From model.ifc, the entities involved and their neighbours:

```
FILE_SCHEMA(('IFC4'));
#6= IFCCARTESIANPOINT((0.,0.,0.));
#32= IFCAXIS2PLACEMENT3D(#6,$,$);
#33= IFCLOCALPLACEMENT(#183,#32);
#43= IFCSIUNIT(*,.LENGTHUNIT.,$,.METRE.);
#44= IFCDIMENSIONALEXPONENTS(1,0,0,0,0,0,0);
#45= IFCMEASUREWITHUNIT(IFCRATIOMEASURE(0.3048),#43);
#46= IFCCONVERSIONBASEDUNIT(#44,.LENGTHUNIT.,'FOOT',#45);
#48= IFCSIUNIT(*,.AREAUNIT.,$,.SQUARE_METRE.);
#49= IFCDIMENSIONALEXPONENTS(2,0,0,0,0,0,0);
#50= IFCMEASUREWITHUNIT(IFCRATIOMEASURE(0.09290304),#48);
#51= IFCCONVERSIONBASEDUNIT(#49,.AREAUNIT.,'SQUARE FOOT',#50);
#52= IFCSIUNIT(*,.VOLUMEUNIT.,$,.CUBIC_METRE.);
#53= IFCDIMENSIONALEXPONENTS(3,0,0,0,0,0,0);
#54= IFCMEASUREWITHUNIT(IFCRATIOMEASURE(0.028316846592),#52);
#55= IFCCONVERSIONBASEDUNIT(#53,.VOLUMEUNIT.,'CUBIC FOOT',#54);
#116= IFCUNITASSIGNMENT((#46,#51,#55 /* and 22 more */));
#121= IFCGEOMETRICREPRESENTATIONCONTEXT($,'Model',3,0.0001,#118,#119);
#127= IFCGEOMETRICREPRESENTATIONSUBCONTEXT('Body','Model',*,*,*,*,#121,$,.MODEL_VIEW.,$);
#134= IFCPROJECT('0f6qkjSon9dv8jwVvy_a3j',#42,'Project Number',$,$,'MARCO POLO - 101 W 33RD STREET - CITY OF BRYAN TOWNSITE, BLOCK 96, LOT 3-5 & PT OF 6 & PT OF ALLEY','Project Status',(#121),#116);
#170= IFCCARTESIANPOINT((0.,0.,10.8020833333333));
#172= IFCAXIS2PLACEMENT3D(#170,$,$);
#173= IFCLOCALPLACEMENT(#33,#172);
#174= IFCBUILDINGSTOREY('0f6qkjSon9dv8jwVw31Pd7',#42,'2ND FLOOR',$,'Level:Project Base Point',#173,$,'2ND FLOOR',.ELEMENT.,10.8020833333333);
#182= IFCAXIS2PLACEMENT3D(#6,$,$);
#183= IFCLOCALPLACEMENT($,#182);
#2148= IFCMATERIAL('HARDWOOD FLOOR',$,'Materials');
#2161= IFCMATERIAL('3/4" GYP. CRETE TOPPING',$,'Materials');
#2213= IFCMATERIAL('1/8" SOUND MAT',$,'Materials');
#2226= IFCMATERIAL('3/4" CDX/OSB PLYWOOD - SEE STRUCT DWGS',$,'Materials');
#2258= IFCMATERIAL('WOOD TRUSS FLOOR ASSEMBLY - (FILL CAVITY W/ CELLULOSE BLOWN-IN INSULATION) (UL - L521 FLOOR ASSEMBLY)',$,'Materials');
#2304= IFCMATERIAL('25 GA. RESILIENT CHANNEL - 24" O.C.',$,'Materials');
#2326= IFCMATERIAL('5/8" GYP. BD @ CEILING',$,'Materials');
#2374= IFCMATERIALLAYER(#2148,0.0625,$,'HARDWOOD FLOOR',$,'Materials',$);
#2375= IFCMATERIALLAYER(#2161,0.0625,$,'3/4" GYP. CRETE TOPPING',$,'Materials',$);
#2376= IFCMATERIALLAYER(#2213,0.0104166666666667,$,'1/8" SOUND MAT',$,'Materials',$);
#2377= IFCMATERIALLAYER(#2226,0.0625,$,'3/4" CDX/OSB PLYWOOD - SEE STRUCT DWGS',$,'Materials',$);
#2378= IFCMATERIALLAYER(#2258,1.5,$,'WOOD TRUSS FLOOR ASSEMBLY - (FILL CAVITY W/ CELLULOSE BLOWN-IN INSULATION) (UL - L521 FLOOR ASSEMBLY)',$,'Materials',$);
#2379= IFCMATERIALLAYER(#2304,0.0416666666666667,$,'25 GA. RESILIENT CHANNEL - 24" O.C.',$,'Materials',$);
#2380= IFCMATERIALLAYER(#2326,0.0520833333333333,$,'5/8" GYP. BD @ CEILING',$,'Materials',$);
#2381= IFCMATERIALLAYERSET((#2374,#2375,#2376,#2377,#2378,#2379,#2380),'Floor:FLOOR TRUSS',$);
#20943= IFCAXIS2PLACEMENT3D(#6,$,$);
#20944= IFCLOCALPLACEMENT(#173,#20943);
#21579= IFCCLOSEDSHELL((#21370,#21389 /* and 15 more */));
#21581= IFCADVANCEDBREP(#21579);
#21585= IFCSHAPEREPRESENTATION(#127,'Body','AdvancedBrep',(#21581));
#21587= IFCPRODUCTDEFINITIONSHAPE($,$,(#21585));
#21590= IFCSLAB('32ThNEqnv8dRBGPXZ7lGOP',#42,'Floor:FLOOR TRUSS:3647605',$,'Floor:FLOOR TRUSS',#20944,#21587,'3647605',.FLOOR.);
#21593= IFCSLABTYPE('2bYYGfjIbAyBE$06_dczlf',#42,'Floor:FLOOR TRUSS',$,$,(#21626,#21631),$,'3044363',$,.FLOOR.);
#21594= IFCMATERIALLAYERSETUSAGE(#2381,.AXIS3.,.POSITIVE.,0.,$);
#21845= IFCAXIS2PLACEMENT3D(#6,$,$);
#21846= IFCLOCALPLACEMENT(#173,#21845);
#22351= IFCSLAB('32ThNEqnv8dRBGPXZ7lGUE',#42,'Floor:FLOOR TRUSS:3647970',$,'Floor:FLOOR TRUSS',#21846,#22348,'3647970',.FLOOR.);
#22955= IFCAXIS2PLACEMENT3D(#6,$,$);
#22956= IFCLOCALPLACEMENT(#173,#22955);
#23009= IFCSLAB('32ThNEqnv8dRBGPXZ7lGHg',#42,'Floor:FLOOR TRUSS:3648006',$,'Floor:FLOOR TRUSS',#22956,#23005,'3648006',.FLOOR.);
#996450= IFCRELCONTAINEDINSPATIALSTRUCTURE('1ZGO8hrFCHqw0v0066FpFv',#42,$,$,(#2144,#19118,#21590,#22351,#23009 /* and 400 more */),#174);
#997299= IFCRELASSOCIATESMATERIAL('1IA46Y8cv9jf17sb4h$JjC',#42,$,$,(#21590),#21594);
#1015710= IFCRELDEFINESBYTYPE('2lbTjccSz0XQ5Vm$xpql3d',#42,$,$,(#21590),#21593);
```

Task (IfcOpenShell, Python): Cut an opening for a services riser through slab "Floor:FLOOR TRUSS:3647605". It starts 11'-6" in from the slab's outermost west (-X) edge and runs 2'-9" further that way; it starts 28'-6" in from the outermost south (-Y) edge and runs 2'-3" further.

```python
import numpy as np
import ifcopenshell
import ifcopenshell.api.feature
import ifcopenshell.api.geometry
import ifcopenshell.api.root
import ifcopenshell.geom
import ifcopenshell.util.placement
import ifcopenshell.util.representation
import ifcopenshell.util.shape
import ifcopenshell.util.unit

model = ifcopenshell.open("model.ifc")
unit_scale = ifcopenshell.util.unit.calculate_unit_scale(model)
settings = ifcopenshell.geom.settings()


def volume(element):
    """Net volume in cubic metres, openings subtracted."""
    shape = ifcopenshell.geom.create_shape(settings, element)
    return ifcopenshell.util.shape.get_volume(shape.geometry)


slab = model.by_guid("32ThNEqnv8dRBGPXZ7lGOP")
before = volume(slab)

# Extent in the slab's own axes, in metres. The edges named are its -X and -Y sides.
slab_shape = ifcopenshell.geom.create_shape(settings, slab)
vertices = ifcopenshell.util.shape.get_vertices(slab_shape.geometry)
x_min, y_min, bottom = vertices.min(axis=0)
top = vertices[:, 2].max()

opening = ifcopenshell.api.root.create_entity(model, ifc_class="IfcOpeningElement", name="Services riser opening", predefined_type="OPENING")
context = ifcopenshell.util.representation.get_context(model, "Model", "Body", "MODEL_VIEW")
width, depth = 0.8382, 0.6858
outline = [(0.0, 0.0), (width, 0.0), (width, depth), (0.0, depth), (0.0, 0.0)]
# Overshoot both faces by 50 mm so the cut is clean.
shape = ifcopenshell.api.geometry.add_slab_representation(
    model, context=context, depth=top - bottom + 0.1, polyline=outline
)
ifcopenshell.api.geometry.assign_representation(model, product=opening, representation=shape)

matrix = ifcopenshell.util.placement.get_local_placement(slab.ObjectPlacement)
matrix[:, 3] = matrix @ np.append(np.array([x_min + 3.5052, y_min + 8.6868, bottom - 0.05]) / unit_scale, 1.0)
ifcopenshell.api.geometry.edit_object_placement(model, product=opening, matrix=matrix, is_si=False)
ifcopenshell.api.feature.add_feature(model, feature=opening, element=slab)

after = volume(slab)

print(f"slab volume {before:.3f} -> {after:.3f} m3")

model.write("model_updated.ifc")
```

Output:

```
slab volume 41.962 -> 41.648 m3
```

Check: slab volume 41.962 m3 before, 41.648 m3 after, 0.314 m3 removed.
